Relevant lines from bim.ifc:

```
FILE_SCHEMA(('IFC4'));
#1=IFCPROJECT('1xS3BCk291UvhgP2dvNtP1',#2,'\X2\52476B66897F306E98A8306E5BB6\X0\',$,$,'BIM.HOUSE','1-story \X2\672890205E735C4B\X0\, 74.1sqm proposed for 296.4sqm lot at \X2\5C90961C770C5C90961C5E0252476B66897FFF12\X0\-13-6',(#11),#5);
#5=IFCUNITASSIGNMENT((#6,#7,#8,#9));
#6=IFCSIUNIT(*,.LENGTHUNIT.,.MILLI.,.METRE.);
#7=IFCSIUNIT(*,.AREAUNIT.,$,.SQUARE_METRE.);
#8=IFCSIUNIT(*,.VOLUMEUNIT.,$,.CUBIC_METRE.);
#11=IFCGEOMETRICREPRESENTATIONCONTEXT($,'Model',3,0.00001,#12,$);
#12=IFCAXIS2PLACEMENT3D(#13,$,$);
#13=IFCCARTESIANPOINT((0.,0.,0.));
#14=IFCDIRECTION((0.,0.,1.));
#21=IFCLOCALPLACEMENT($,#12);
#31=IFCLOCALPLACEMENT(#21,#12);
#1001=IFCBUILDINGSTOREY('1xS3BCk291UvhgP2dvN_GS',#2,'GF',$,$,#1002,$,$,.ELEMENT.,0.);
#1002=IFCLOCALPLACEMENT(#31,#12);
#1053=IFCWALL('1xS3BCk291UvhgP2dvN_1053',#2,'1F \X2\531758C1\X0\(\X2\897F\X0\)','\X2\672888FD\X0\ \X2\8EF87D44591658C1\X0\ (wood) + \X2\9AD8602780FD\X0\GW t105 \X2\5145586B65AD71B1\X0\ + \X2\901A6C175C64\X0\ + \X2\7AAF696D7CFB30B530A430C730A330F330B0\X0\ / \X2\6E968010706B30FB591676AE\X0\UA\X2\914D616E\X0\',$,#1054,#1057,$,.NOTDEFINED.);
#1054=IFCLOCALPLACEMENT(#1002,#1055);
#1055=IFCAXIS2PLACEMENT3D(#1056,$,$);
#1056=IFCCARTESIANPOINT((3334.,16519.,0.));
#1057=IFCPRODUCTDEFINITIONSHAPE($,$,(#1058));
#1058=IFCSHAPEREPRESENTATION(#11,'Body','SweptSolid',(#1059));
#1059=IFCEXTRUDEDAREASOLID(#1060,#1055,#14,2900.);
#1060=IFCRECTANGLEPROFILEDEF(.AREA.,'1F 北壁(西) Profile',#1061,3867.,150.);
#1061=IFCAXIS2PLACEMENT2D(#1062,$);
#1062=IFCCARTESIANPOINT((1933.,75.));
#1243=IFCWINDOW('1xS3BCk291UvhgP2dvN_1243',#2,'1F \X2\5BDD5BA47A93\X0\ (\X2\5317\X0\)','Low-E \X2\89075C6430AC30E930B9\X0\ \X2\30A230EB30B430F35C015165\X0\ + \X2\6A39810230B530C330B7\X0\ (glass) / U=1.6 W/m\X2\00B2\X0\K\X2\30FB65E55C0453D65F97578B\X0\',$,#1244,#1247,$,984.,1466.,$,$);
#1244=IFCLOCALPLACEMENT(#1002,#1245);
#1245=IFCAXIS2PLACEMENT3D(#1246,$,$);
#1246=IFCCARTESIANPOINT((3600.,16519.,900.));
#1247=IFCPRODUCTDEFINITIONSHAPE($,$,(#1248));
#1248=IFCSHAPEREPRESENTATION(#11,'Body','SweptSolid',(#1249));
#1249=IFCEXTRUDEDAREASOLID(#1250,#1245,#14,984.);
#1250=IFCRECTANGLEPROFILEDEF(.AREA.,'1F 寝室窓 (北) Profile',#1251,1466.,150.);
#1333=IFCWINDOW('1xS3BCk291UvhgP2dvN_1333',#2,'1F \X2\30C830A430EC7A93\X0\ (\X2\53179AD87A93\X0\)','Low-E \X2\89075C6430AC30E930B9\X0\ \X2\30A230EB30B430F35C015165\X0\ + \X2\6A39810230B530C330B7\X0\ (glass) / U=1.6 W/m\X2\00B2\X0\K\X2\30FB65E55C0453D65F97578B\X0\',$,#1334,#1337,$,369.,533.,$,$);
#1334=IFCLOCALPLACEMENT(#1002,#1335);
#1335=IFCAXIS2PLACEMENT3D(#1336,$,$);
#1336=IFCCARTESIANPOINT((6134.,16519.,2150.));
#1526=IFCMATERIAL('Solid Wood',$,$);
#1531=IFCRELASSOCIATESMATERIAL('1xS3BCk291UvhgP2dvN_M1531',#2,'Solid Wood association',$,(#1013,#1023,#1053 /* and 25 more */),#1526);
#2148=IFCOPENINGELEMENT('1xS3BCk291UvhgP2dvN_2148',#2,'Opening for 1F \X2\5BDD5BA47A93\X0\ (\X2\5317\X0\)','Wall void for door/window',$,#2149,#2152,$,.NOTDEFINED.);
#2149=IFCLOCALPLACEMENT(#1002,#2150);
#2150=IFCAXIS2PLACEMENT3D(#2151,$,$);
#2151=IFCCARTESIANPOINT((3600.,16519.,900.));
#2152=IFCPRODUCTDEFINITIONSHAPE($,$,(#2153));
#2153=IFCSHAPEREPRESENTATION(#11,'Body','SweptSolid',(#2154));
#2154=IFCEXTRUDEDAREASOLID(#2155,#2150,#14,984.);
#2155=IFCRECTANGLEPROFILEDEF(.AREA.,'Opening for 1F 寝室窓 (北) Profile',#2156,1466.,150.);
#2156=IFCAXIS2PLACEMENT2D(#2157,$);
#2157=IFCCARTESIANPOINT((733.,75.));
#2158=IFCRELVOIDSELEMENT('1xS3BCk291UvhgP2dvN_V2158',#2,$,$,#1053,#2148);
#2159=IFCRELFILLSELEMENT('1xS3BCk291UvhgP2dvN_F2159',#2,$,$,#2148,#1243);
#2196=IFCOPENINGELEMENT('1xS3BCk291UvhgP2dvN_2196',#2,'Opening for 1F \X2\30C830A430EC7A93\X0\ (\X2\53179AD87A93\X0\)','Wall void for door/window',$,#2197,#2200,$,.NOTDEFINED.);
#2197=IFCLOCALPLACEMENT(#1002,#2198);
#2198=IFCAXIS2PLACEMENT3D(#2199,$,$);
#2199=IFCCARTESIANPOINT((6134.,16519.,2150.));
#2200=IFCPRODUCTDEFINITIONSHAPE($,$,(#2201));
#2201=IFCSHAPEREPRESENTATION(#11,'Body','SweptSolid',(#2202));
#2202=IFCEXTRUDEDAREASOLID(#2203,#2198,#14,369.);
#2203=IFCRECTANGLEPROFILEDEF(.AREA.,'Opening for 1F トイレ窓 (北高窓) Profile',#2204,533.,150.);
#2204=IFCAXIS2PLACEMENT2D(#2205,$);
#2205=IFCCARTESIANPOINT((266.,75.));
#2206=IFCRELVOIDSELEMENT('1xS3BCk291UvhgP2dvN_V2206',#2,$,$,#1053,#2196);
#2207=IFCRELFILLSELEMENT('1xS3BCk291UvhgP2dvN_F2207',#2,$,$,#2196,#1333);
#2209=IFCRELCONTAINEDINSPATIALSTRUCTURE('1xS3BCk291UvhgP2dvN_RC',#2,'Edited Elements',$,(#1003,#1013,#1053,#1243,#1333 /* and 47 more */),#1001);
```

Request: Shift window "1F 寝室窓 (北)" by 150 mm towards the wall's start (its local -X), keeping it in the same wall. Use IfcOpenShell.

```python
import ifcopenshell
import ifcopenshell.api.geometry
import ifcopenshell.util.placement

model = ifcopenshell.open("bim.ifc")

window = model.by_guid("1xS3BCk291UvhgP2dvN_1243")
opening = window.FillsVoids[0].RelatingOpeningElement
wall = opening.VoidsElements[0].RelatingBuildingElement

wall_matrix = ifcopenshell.util.placement.get_local_placement(wall.ObjectPlacement)
shift = wall_matrix[:3, 0] * -150.0
before = ifcopenshell.util.placement.get_local_placement(window.ObjectPlacement)[:3, 3].copy()

# The window is not placed relative to its opening, so move both.
for product in (opening, window):
    matrix = ifcopenshell.util.placement.get_local_placement(product.ObjectPlacement)
    matrix[:3, 3] += shift
    ifcopenshell.api.geometry.edit_object_placement(model, product=product, matrix=matrix, is_si=False)

after = ifcopenshell.util.placement.get_local_placement(window.ObjectPlacement)[:3, 3]
print("window moved by", (after - before).round(3) + 0.0)

model.write("bim-out.ifc")
```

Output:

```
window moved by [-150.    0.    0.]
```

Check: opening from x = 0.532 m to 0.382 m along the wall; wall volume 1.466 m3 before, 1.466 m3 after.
